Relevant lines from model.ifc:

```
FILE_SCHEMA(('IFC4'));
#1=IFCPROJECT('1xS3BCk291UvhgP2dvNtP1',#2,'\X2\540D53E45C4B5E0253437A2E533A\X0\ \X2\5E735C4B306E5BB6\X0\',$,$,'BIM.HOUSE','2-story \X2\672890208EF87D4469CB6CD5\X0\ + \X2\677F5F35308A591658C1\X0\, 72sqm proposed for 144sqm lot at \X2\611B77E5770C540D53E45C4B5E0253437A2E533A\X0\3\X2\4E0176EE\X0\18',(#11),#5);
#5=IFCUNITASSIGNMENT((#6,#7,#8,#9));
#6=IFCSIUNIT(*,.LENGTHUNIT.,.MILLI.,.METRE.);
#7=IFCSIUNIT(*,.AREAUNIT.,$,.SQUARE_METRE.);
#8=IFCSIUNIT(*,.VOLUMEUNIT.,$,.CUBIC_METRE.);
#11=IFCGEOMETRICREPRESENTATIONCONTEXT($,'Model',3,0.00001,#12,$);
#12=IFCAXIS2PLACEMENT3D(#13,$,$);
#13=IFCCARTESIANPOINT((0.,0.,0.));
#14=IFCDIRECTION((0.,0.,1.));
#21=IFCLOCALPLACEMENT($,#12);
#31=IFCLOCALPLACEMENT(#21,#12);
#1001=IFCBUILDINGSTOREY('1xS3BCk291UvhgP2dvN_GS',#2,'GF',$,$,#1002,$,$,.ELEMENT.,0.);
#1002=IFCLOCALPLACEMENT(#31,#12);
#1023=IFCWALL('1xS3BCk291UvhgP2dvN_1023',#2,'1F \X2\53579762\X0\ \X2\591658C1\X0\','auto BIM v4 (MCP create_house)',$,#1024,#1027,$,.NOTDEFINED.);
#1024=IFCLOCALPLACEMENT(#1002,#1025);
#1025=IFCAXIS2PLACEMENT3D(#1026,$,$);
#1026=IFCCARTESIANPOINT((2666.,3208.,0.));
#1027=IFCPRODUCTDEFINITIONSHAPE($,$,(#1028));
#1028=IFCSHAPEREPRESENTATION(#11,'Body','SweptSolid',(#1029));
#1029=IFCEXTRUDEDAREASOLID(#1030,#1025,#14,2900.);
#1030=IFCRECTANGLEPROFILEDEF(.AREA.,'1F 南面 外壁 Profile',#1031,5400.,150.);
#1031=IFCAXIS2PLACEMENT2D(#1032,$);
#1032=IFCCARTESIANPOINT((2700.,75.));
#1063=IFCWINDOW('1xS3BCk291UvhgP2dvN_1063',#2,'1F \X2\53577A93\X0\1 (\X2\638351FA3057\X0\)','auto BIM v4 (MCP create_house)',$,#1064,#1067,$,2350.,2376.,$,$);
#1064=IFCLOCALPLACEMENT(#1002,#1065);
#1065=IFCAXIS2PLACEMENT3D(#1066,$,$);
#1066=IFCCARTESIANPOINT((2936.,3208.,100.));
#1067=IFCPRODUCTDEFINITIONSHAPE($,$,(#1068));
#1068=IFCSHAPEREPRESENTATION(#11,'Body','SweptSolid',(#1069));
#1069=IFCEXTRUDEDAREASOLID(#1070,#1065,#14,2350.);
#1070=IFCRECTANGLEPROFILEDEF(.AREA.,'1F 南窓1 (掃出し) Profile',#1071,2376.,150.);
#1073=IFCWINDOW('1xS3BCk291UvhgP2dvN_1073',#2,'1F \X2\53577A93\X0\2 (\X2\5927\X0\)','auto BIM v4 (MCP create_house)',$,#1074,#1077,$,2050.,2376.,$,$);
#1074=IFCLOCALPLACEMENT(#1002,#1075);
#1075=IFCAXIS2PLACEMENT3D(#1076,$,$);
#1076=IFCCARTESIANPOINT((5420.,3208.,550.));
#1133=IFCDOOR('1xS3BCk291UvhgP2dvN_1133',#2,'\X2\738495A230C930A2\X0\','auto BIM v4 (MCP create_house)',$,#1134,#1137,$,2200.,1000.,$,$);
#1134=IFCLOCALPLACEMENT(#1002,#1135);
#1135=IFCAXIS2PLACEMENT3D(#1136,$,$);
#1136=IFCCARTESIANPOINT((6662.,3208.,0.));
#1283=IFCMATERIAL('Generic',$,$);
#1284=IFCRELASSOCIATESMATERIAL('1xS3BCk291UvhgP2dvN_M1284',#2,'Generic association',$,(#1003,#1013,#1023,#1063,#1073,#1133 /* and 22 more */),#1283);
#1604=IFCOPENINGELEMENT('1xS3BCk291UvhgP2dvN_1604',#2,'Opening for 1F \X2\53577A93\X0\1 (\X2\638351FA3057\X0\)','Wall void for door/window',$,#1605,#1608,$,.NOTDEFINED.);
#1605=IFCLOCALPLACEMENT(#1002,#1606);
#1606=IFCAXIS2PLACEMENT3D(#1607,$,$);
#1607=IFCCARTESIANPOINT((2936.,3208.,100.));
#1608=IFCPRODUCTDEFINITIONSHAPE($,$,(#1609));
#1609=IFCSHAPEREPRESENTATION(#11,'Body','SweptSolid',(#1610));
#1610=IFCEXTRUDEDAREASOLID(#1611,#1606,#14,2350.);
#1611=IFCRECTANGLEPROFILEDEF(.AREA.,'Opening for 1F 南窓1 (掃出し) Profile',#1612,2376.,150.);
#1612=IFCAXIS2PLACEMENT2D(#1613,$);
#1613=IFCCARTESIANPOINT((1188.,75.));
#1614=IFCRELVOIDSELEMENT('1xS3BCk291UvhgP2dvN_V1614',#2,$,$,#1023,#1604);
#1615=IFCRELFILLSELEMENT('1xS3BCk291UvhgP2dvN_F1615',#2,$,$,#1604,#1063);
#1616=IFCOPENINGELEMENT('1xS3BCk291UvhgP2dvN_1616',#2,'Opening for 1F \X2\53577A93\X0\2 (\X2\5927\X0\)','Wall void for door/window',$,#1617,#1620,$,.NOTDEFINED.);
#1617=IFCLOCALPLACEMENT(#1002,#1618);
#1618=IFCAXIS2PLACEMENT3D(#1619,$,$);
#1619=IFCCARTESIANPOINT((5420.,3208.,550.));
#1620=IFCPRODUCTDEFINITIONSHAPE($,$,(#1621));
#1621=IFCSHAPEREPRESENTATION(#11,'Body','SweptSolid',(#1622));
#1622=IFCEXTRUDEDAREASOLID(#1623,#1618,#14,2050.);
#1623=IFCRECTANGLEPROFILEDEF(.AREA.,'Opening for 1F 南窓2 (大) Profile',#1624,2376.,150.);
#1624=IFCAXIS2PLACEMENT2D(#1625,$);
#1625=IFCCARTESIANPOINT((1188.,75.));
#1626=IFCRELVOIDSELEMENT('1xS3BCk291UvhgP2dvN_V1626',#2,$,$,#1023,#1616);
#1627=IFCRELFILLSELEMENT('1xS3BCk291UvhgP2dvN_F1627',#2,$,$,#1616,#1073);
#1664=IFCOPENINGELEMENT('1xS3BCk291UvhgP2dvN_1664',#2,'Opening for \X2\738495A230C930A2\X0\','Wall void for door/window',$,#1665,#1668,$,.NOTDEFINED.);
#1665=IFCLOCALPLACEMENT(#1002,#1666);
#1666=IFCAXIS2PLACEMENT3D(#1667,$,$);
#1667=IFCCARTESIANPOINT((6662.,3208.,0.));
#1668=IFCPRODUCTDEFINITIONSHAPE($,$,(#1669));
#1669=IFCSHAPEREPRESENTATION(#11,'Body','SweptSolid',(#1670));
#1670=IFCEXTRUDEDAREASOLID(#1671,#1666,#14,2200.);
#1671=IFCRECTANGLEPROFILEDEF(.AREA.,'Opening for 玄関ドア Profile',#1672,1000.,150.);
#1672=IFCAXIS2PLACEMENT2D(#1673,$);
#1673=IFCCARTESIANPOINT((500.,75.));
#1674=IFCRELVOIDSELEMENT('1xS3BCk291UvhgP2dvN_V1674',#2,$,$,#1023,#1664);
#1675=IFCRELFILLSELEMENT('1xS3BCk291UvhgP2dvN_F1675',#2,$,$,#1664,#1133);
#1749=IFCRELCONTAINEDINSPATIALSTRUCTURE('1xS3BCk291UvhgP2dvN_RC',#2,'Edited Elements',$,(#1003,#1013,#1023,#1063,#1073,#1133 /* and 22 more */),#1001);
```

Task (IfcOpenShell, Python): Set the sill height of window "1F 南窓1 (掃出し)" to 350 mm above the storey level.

```python
import numpy as np
import ifcopenshell
import ifcopenshell.api.geometry
import ifcopenshell.geom
import ifcopenshell.util.element
import ifcopenshell.util.placement
import ifcopenshell.util.shape
import ifcopenshell.util.unit

model = ifcopenshell.open("model.ifc")
unit_scale = ifcopenshell.util.unit.calculate_unit_scale(model)

window = model.by_guid("1xS3BCk291UvhgP2dvN_1063")
opening = window.FillsVoids[0].RelatingOpeningElement
storey = ifcopenshell.util.element.get_container(window, ifc_class="IfcBuildingStorey")
level = ifcopenshell.util.placement.get_local_placement(storey.ObjectPlacement)[2, 3]

# The opening's origin need not be at the sill, so measure its lowest point.
shape = ifcopenshell.geom.create_shape(ifcopenshell.geom.settings(), opening)
bottom = ifcopenshell.util.shape.get_shape_bottom_elevation(shape, shape.geometry) / unit_scale
dz = level + 0.35 / unit_scale - bottom

shift = np.array([0.0, 0.0, dz])
# The window is not placed relative to its opening, so move both.
for product in (opening, window):
    matrix = ifcopenshell.util.placement.get_local_placement(product.ObjectPlacement)
    matrix[:3, 3] += shift
    ifcopenshell.api.geometry.edit_object_placement(model, product=product, matrix=matrix, is_si=False)

print(f"moved by {dz * unit_scale:+.3f} m")

model.write("model_v2.ifc")
```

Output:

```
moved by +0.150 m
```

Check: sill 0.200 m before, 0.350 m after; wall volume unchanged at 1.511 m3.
